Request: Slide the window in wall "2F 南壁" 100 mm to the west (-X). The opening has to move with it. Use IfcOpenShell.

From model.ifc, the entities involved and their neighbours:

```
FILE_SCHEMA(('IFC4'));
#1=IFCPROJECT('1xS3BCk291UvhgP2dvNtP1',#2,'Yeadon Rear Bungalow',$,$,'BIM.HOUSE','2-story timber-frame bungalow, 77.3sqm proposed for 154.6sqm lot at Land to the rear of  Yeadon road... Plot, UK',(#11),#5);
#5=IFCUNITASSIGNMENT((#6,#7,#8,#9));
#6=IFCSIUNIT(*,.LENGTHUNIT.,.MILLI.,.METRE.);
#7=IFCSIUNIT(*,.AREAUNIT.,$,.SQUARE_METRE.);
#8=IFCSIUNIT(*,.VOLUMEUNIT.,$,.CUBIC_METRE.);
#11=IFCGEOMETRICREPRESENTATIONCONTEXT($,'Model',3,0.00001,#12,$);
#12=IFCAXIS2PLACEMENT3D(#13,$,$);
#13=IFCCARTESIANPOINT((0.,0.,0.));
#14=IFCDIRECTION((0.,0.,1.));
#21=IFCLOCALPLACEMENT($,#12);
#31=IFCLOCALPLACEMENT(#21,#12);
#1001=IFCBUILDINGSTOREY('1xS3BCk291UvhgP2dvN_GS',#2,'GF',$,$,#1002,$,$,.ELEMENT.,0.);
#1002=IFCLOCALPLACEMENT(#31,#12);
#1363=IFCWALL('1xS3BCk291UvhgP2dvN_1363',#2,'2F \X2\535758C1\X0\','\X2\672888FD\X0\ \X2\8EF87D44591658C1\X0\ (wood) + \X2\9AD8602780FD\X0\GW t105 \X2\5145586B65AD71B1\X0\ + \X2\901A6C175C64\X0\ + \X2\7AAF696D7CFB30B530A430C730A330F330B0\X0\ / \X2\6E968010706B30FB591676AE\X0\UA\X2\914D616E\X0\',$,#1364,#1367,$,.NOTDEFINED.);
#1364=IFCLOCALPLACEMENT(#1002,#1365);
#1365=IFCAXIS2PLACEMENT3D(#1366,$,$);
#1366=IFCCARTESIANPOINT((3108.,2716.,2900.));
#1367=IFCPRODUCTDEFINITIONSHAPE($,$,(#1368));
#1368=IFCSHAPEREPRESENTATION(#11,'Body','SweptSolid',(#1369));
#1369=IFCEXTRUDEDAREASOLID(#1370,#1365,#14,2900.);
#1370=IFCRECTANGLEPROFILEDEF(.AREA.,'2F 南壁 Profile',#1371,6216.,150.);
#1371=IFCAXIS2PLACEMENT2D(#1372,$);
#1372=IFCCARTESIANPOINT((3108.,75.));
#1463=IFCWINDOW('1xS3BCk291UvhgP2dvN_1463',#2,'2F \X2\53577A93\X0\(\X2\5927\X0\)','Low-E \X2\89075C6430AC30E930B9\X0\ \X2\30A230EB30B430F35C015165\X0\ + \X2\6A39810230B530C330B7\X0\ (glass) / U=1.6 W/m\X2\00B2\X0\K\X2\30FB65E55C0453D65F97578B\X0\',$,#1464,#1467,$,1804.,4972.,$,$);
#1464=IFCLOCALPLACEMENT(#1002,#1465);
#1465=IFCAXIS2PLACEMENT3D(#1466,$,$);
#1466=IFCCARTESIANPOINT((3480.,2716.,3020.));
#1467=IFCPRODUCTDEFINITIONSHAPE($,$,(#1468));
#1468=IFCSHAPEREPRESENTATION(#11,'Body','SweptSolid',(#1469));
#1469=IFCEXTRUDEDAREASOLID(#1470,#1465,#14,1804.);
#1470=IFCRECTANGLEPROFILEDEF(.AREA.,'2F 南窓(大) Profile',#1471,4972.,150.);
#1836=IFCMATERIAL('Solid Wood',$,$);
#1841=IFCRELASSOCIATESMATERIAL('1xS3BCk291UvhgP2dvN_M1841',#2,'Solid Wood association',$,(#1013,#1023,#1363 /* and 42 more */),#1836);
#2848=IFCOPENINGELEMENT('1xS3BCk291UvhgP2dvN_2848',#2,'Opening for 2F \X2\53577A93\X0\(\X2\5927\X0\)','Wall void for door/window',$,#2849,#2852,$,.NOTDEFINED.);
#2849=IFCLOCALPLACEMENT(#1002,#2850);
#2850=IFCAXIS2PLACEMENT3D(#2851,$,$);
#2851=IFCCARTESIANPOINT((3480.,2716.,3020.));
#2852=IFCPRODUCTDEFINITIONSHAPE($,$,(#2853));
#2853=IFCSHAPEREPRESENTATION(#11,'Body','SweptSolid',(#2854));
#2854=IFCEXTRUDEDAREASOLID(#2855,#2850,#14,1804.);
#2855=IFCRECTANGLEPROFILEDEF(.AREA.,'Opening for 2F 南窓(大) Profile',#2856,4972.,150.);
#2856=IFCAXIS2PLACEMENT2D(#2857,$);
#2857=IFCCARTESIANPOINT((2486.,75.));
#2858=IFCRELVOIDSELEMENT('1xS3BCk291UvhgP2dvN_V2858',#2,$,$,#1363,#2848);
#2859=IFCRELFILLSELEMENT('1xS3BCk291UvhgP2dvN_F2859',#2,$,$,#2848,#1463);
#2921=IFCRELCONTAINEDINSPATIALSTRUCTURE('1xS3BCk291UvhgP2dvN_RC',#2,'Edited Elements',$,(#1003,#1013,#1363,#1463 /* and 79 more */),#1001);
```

```python
import ifcopenshell
import ifcopenshell.api.geometry
import ifcopenshell.util.placement
import ifcopenshell.util.unit

model = ifcopenshell.open("model.ifc")
unit_scale = ifcopenshell.util.unit.calculate_unit_scale(model)

window = model.by_guid("1xS3BCk291UvhgP2dvN_1463")
opening = window.FillsVoids[0].RelatingOpeningElement
wall = opening.VoidsElements[0].RelatingBuildingElement

wall_matrix = ifcopenshell.util.placement.get_local_placement(wall.ObjectPlacement)
shift = wall_matrix[:3, 0] * -0.1 / unit_scale
before = ifcopenshell.util.placement.get_local_placement(window.ObjectPlacement)[:3, 3].copy()

# The window is not placed relative to its opening, so move both.
for product in (opening, window):
    matrix = ifcopenshell.util.placement.get_local_placement(product.ObjectPlacement)
    matrix[:3, 3] += shift
    ifcopenshell.api.geometry.edit_object_placement(model, product=product, matrix=matrix, is_si=False)

after = ifcopenshell.util.placement.get_local_placement(window.ObjectPlacement)[:3, 3]
print("window moved by", (after - before).round(3) + 0.0)

model.write("model_rev.ifc")
```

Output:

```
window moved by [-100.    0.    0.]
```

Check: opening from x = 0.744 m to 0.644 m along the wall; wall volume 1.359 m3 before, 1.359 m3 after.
